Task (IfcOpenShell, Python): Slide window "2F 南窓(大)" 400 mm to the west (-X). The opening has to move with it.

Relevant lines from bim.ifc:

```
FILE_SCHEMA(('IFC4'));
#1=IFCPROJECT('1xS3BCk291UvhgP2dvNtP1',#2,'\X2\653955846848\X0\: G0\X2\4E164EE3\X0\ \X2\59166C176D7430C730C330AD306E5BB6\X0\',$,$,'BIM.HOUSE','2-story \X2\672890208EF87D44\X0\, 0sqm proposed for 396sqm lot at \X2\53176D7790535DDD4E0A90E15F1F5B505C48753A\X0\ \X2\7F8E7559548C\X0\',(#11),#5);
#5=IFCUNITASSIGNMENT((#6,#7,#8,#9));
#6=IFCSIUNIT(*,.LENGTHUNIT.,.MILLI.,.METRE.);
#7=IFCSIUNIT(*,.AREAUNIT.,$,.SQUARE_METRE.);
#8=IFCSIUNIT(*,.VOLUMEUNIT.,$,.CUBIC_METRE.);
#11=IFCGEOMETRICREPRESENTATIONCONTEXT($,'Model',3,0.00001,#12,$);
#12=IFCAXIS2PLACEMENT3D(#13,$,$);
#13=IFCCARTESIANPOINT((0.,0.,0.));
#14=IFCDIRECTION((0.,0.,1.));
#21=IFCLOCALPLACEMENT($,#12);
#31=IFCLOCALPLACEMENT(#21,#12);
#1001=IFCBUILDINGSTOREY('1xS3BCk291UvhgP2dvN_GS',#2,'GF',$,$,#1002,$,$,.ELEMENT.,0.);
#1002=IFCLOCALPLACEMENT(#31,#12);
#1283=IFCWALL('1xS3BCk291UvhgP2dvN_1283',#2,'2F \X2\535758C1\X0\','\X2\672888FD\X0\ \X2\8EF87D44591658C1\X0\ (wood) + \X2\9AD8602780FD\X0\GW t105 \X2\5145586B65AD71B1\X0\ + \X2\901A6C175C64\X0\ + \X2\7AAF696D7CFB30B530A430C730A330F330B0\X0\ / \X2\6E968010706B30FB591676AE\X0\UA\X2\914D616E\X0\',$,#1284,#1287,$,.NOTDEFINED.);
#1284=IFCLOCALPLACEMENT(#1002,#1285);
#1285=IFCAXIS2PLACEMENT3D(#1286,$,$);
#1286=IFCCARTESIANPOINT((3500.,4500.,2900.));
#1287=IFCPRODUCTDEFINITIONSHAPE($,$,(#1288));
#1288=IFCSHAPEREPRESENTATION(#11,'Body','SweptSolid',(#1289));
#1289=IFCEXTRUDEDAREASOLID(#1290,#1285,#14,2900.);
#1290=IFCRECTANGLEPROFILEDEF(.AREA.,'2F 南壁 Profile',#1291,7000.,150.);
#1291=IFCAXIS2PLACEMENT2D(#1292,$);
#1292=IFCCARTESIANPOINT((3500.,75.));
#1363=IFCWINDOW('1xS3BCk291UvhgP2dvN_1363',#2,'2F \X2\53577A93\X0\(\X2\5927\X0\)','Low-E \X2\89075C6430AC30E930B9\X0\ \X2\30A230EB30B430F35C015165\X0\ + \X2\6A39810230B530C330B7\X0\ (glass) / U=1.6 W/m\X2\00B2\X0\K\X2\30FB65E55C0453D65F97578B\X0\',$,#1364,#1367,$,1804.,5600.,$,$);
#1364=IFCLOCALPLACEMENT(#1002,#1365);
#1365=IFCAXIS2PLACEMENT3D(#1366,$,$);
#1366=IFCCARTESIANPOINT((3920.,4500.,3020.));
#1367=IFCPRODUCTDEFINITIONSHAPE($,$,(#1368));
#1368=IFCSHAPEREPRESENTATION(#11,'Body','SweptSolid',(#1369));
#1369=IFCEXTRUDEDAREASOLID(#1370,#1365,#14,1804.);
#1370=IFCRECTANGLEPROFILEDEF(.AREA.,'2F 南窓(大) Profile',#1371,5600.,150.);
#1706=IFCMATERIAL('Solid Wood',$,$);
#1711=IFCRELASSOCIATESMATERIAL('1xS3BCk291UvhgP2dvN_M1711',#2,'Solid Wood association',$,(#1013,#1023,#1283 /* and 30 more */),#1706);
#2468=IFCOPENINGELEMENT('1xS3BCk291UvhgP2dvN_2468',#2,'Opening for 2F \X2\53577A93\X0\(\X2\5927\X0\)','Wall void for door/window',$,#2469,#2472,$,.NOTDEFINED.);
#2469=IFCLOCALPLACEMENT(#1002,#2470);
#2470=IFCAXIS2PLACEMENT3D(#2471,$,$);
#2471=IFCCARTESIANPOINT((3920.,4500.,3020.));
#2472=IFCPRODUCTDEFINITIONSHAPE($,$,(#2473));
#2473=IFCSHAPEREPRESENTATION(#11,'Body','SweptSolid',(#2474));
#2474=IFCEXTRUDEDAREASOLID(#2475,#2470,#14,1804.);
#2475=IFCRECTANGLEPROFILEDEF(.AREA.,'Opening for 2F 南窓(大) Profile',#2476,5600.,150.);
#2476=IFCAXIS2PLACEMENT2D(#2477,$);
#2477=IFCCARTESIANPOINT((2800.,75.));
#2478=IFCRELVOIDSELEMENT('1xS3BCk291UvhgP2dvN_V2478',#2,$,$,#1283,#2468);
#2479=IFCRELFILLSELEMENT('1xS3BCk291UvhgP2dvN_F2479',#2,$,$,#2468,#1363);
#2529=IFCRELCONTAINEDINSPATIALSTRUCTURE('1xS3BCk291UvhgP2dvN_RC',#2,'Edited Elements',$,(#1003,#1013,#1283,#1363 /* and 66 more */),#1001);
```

```python
import ifcopenshell
import ifcopenshell.api.geometry
import ifcopenshell.util.placement

model = ifcopenshell.open("bim.ifc")

window = model.by_guid("1xS3BCk291UvhgP2dvN_1363")
opening = window.FillsVoids[0].RelatingOpeningElement
wall = opening.VoidsElements[0].RelatingBuildingElement

wall_matrix = ifcopenshell.util.placement.get_local_placement(wall.ObjectPlacement)
shift = wall_matrix[:3, 0] * -400.0
before = ifcopenshell.util.placement.get_local_placement(window.ObjectPlacement)[:3, 3].copy()

# The window is not placed relative to its opening, so move both.
for product in (opening, window):
    matrix = ifcopenshell.util.placement.get_local_placement(product.ObjectPlacement)
    matrix[:3, 3] += shift
    ifcopenshell.api.geometry.edit_object_placement(model, product=product, matrix=matrix, is_si=False)

after = ifcopenshell.util.placement.get_local_placement(window.ObjectPlacement)[:3, 3]
print("window moved by", (after - before).round(3) + 0.0)

model.write("bim_rev.ifc")
```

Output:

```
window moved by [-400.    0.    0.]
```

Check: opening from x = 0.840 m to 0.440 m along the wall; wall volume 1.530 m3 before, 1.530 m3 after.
